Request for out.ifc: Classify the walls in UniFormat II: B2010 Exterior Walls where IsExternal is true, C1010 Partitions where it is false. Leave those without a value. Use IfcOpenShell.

First a look at what the model holds.

```python
import ifcopenshell
import ifcopenshell.util.element

model = ifcopenshell.open("out.ifc")
print(model.schema)
print("classifications:", [c.Name for c in model.by_type("IfcClassification")])
values = [ifcopenshell.util.element.get_pset(e, "Pset_WallCommon", "IsExternal") for e in model.by_type("IfcWall")]
for value in (True, False, None):
    print("IsExternal", value, values.count(value))
```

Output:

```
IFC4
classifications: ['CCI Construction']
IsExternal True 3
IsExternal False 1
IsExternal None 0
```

```python
import ifcopenshell
import ifcopenshell.api.classification
import ifcopenshell.util.element

model = ifcopenshell.open("out.ifc")

system = ifcopenshell.api.classification.add_classification(model, classification="UniFormat II")

walls = model.by_type("IfcWall")
external = {e: ifcopenshell.util.element.get_pset(e, "Pset_WallCommon", "IsExternal") for e in walls}
for flag, code, name in ((True, "B2010", "Exterior Walls"), (False, "C1010", "Partitions")):
    products = [e for e in walls if external[e] is flag]
    ifcopenshell.api.classification.add_reference(
        model, products=products, classification=system, identification=code, name=name
    )
    print(code, len(products))

model.write("out_updated.ifc")
```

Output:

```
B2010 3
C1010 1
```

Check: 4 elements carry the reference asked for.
